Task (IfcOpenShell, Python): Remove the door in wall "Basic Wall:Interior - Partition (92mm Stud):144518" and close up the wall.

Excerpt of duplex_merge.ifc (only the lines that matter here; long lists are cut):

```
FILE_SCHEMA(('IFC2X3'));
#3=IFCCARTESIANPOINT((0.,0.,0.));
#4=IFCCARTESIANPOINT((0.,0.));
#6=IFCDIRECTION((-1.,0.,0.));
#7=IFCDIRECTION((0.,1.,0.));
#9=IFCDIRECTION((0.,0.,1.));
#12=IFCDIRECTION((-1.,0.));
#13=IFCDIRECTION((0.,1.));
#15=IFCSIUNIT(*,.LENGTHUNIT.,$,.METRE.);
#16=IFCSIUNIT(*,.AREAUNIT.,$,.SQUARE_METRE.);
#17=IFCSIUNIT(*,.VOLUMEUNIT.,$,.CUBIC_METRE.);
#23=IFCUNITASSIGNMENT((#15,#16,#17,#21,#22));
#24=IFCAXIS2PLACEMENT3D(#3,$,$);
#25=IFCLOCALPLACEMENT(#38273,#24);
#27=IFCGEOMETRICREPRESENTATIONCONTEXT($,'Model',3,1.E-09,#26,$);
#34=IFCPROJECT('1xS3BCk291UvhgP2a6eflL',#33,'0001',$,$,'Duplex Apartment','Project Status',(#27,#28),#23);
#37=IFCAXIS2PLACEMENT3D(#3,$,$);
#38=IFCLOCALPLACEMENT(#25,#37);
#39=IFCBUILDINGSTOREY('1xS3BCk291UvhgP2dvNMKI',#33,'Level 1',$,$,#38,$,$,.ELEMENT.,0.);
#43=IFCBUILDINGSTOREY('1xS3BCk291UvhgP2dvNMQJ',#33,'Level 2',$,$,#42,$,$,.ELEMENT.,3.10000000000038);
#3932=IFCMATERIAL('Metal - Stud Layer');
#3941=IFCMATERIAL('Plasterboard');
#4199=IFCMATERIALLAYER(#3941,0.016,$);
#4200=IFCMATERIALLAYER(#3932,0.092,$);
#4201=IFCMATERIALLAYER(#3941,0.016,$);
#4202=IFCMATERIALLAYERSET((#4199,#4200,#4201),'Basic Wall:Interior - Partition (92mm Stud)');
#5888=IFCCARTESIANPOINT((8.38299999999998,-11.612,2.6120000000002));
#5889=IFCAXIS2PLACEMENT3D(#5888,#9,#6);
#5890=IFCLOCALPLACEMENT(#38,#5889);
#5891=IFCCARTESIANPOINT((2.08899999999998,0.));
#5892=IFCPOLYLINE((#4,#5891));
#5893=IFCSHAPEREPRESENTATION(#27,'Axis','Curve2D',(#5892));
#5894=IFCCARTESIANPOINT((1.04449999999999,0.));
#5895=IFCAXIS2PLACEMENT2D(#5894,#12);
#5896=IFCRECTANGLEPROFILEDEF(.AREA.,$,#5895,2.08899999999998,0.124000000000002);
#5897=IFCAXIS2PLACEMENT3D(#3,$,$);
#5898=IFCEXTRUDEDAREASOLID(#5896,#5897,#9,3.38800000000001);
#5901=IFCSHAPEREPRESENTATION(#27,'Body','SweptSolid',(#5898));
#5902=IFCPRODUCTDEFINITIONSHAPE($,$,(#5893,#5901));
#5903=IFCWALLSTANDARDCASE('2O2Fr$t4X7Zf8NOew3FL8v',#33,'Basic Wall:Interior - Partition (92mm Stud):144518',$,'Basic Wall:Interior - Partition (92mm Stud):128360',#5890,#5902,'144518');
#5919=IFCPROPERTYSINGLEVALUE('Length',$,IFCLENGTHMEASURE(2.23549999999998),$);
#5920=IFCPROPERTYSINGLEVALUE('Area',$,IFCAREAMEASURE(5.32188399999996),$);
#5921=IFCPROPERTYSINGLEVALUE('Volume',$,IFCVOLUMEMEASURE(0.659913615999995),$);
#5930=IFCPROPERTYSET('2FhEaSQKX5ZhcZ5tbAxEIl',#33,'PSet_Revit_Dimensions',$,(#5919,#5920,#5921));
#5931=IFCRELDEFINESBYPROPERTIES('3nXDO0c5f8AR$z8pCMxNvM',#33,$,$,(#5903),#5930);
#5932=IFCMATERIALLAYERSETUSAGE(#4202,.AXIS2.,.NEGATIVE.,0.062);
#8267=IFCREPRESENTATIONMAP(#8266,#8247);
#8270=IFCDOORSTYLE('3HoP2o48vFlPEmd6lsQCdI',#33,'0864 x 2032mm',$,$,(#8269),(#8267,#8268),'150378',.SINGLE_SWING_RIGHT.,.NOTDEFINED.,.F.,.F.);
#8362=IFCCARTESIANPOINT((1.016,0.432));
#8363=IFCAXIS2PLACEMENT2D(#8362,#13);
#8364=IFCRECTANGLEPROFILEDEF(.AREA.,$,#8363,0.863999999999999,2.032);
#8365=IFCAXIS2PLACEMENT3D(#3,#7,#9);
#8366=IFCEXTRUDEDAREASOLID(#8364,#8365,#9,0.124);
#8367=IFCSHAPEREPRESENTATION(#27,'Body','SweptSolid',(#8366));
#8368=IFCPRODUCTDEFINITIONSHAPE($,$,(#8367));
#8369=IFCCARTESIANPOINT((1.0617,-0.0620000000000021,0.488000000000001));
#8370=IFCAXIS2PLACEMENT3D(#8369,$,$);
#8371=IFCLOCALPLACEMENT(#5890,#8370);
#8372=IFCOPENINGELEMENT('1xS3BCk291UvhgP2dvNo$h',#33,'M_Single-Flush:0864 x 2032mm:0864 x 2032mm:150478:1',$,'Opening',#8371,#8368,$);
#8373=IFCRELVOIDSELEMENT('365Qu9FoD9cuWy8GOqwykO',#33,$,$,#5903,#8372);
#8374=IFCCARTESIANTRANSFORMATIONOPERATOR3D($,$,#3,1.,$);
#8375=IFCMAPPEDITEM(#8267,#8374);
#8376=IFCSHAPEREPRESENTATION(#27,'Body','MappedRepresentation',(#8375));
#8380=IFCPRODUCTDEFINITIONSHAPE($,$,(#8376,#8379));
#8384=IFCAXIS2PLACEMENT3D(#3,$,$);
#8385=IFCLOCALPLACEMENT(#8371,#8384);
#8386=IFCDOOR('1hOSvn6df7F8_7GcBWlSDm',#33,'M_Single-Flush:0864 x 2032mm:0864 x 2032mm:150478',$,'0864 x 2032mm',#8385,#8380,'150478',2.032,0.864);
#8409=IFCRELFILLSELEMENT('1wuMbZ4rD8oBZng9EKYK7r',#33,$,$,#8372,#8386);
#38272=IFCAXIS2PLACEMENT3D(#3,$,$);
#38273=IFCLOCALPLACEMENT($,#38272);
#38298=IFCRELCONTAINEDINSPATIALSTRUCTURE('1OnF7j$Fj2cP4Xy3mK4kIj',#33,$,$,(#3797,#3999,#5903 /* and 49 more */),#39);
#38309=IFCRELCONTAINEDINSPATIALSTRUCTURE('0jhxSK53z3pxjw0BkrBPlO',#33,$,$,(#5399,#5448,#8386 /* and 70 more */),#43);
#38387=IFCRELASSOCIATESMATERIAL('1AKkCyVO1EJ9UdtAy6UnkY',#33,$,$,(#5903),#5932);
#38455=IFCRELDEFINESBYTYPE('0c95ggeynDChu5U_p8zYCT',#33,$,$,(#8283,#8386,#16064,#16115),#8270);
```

```python
import ifcopenshell
import ifcopenshell.api.feature
import ifcopenshell.api.pset
import ifcopenshell.api.root
import ifcopenshell.geom
import ifcopenshell.util.element
import ifcopenshell.util.shape
import ifcopenshell.util.unit

model = ifcopenshell.open("duplex_merge.ifc")
area_scale = ifcopenshell.util.unit.calculate_unit_scale(model, "AREAUNIT")
volume_scale = ifcopenshell.util.unit.calculate_unit_scale(model, "VOLUMEUNIT")
settings = ifcopenshell.geom.settings()


def volume(element):
    """Net volume in cubic metres, openings subtracted."""
    shape = ifcopenshell.geom.create_shape(settings, element)
    return ifcopenshell.util.shape.get_volume(shape.geometry)


door = model.by_id(8386)
opening = door.FillsVoids[0].RelatingOpeningElement
wall = opening.VoidsElements[0].RelatingBuildingElement
before = volume(wall)

ifcopenshell.api.root.remove_product(model, product=door)
ifcopenshell.api.feature.remove_feature(model, feature=opening)

after = volume(wall)
thickness = 0.124  # wall thickness in metres

# Update the wall's stored quantities.
pset = model.by_id(ifcopenshell.util.element.get_pset(wall, "PSet_Revit_Dimensions", should_inherit=False)["id"])
ifcopenshell.api.pset.edit_pset(model, pset=pset, properties={
    "Area": model.create_entity("IfcAreaMeasure", after / thickness / area_scale),
    "Volume": model.create_entity("IfcVolumeMeasure", after / volume_scale),
})

print(f"wall volume {before:.3f} -> {after:.3f} m3")

model.write("duplex_merge_v2.ifc")
```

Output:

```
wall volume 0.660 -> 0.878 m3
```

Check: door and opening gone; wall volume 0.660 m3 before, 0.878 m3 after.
